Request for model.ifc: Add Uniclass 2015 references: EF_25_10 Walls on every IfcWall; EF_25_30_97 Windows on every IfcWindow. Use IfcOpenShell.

First a look at what the model holds.

```python
import ifcopenshell

model = ifcopenshell.open("model.ifc")
print(model.schema)
print("classifications:", [c.Name for c in model.by_type("IfcClassification")])
for ifc_class in ("IfcDoor", "IfcRoof", "IfcStair", "IfcWall", "IfcWindow"):
    print(ifc_class, len(model.by_type(ifc_class)))
```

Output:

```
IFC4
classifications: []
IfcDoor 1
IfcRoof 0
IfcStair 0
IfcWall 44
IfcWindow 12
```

```python
import ifcopenshell
import ifcopenshell.api.classification

model = ifcopenshell.open("model.ifc")

system = ifcopenshell.api.classification.add_classification(model, classification="Uniclass 2015")

codes = {
    "IfcWall": ("EF_25_10", "Walls"),
    "IfcWindow": ("EF_25_30_97", "Windows"),
}
for ifc_class, (code, name) in codes.items():
    products = model.by_type(ifc_class)
    ifcopenshell.api.classification.add_reference(
        model, products=products, classification=system, identification=code, name=name
    )
    print(code, len(products))

model.write("model_v2.ifc")
```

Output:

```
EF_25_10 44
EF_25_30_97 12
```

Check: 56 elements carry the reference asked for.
